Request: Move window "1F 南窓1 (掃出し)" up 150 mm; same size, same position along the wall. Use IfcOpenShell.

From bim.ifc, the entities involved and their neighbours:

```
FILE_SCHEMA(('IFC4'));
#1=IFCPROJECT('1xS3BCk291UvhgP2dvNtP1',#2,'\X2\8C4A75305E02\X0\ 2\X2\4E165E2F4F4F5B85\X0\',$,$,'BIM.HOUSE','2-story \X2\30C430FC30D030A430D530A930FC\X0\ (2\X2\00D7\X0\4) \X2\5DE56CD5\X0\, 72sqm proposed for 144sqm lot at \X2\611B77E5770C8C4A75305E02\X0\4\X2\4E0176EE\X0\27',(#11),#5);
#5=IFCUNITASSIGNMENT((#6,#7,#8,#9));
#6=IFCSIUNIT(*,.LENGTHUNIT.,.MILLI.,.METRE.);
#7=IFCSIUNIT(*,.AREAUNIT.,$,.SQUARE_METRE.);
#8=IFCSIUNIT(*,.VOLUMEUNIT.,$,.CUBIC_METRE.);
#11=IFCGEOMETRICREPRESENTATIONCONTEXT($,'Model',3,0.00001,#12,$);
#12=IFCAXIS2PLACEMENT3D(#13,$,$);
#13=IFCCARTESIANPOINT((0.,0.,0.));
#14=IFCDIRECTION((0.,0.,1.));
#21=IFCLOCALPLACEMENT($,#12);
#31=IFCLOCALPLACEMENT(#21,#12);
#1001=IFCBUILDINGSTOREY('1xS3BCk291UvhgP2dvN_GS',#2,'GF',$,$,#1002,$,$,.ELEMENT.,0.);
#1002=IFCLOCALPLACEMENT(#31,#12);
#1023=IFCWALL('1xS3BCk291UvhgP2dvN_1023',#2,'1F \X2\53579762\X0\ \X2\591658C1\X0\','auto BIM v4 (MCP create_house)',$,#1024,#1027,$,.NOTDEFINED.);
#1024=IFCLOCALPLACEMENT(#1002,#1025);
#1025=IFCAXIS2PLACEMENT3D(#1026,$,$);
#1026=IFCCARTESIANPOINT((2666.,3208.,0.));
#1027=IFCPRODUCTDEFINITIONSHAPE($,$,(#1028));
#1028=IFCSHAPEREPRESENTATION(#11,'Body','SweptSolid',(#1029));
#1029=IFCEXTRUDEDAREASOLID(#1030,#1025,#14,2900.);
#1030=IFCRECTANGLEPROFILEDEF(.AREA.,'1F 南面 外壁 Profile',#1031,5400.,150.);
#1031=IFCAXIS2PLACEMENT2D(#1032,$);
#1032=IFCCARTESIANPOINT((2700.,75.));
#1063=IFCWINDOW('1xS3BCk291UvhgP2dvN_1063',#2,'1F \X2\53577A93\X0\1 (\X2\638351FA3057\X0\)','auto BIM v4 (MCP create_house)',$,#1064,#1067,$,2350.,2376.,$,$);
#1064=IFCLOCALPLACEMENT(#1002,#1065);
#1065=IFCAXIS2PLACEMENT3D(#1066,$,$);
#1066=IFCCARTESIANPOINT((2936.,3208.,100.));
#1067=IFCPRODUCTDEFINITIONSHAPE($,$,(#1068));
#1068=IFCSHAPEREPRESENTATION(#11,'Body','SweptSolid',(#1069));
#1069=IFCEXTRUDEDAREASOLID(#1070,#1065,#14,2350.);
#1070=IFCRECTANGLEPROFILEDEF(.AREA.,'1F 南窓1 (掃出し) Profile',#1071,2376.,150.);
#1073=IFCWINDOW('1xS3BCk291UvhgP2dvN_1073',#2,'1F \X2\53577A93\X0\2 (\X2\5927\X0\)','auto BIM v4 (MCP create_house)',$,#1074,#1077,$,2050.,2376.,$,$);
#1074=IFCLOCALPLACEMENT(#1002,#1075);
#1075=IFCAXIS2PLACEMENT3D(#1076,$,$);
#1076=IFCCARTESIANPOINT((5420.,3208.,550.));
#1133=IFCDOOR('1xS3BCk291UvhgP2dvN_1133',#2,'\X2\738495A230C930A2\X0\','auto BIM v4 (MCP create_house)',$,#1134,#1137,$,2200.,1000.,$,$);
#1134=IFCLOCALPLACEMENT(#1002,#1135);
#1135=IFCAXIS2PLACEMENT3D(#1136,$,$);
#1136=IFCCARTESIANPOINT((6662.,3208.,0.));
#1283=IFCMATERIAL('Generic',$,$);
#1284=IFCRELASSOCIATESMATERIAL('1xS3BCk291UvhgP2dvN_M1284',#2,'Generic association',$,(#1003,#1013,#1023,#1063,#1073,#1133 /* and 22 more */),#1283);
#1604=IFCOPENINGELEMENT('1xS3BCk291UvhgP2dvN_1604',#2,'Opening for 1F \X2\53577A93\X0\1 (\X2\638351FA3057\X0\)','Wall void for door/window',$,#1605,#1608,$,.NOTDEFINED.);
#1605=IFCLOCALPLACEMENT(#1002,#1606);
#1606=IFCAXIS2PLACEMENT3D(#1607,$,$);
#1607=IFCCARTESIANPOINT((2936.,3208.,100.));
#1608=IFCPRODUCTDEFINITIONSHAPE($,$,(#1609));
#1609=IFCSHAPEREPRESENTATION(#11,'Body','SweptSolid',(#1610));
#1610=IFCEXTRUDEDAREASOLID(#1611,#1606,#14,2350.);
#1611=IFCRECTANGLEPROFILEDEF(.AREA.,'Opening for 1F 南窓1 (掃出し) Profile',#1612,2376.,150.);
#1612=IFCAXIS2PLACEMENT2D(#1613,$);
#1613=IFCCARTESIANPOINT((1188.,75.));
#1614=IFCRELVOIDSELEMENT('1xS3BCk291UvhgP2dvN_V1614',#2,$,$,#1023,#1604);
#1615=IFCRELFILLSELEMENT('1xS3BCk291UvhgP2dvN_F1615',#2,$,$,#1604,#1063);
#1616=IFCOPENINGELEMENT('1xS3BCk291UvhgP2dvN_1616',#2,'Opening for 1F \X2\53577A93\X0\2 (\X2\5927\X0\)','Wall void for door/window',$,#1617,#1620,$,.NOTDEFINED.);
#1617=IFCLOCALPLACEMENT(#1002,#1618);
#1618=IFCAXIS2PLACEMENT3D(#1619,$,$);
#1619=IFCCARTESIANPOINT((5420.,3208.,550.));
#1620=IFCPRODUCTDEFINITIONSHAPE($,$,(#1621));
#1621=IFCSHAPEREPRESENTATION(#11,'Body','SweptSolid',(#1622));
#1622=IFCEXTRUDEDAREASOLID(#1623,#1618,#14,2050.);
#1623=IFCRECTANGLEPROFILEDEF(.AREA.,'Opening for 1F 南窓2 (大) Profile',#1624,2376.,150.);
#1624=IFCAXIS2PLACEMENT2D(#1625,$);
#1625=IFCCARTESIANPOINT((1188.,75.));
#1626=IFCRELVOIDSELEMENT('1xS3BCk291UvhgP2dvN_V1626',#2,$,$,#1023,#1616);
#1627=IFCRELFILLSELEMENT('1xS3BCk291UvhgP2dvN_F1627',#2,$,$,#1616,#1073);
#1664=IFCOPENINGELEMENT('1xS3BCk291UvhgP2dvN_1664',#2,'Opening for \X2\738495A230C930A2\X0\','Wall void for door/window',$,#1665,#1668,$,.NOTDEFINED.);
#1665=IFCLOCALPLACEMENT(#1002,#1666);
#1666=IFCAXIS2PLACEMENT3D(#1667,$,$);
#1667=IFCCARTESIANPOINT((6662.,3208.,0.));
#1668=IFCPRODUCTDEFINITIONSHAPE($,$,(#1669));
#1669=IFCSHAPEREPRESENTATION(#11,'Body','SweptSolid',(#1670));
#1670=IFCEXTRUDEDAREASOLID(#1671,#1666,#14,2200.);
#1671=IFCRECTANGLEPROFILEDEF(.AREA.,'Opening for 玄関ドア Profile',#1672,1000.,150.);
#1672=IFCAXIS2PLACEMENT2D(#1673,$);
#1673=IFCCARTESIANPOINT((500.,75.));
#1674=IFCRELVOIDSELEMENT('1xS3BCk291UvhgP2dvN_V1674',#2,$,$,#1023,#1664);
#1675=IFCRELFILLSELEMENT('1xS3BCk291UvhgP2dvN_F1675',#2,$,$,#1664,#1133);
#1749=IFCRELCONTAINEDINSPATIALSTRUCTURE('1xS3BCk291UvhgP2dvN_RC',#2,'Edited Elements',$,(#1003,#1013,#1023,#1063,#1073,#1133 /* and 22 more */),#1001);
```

```python
import numpy as np
import ifcopenshell
import ifcopenshell.api.geometry
import ifcopenshell.util.placement
import ifcopenshell.util.unit

model = ifcopenshell.open("bim.ifc")
unit_scale = ifcopenshell.util.unit.calculate_unit_scale(model)

window = model.by_guid("1xS3BCk291UvhgP2dvN_1063")
opening = window.FillsVoids[0].RelatingOpeningElement
dz = 0.15 / unit_scale

shift = np.array([0.0, 0.0, dz])
# The window is not placed relative to its opening, so move both.
for product in (opening, window):
    matrix = ifcopenshell.util.placement.get_local_placement(product.ObjectPlacement)
    matrix[:3, 3] += shift
    ifcopenshell.api.geometry.edit_object_placement(model, product=product, matrix=matrix, is_si=False)

print(f"moved by {dz * unit_scale:+.3f} m")

model.write("bim_rev.ifc")
```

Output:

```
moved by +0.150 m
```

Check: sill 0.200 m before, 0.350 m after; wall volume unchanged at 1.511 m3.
